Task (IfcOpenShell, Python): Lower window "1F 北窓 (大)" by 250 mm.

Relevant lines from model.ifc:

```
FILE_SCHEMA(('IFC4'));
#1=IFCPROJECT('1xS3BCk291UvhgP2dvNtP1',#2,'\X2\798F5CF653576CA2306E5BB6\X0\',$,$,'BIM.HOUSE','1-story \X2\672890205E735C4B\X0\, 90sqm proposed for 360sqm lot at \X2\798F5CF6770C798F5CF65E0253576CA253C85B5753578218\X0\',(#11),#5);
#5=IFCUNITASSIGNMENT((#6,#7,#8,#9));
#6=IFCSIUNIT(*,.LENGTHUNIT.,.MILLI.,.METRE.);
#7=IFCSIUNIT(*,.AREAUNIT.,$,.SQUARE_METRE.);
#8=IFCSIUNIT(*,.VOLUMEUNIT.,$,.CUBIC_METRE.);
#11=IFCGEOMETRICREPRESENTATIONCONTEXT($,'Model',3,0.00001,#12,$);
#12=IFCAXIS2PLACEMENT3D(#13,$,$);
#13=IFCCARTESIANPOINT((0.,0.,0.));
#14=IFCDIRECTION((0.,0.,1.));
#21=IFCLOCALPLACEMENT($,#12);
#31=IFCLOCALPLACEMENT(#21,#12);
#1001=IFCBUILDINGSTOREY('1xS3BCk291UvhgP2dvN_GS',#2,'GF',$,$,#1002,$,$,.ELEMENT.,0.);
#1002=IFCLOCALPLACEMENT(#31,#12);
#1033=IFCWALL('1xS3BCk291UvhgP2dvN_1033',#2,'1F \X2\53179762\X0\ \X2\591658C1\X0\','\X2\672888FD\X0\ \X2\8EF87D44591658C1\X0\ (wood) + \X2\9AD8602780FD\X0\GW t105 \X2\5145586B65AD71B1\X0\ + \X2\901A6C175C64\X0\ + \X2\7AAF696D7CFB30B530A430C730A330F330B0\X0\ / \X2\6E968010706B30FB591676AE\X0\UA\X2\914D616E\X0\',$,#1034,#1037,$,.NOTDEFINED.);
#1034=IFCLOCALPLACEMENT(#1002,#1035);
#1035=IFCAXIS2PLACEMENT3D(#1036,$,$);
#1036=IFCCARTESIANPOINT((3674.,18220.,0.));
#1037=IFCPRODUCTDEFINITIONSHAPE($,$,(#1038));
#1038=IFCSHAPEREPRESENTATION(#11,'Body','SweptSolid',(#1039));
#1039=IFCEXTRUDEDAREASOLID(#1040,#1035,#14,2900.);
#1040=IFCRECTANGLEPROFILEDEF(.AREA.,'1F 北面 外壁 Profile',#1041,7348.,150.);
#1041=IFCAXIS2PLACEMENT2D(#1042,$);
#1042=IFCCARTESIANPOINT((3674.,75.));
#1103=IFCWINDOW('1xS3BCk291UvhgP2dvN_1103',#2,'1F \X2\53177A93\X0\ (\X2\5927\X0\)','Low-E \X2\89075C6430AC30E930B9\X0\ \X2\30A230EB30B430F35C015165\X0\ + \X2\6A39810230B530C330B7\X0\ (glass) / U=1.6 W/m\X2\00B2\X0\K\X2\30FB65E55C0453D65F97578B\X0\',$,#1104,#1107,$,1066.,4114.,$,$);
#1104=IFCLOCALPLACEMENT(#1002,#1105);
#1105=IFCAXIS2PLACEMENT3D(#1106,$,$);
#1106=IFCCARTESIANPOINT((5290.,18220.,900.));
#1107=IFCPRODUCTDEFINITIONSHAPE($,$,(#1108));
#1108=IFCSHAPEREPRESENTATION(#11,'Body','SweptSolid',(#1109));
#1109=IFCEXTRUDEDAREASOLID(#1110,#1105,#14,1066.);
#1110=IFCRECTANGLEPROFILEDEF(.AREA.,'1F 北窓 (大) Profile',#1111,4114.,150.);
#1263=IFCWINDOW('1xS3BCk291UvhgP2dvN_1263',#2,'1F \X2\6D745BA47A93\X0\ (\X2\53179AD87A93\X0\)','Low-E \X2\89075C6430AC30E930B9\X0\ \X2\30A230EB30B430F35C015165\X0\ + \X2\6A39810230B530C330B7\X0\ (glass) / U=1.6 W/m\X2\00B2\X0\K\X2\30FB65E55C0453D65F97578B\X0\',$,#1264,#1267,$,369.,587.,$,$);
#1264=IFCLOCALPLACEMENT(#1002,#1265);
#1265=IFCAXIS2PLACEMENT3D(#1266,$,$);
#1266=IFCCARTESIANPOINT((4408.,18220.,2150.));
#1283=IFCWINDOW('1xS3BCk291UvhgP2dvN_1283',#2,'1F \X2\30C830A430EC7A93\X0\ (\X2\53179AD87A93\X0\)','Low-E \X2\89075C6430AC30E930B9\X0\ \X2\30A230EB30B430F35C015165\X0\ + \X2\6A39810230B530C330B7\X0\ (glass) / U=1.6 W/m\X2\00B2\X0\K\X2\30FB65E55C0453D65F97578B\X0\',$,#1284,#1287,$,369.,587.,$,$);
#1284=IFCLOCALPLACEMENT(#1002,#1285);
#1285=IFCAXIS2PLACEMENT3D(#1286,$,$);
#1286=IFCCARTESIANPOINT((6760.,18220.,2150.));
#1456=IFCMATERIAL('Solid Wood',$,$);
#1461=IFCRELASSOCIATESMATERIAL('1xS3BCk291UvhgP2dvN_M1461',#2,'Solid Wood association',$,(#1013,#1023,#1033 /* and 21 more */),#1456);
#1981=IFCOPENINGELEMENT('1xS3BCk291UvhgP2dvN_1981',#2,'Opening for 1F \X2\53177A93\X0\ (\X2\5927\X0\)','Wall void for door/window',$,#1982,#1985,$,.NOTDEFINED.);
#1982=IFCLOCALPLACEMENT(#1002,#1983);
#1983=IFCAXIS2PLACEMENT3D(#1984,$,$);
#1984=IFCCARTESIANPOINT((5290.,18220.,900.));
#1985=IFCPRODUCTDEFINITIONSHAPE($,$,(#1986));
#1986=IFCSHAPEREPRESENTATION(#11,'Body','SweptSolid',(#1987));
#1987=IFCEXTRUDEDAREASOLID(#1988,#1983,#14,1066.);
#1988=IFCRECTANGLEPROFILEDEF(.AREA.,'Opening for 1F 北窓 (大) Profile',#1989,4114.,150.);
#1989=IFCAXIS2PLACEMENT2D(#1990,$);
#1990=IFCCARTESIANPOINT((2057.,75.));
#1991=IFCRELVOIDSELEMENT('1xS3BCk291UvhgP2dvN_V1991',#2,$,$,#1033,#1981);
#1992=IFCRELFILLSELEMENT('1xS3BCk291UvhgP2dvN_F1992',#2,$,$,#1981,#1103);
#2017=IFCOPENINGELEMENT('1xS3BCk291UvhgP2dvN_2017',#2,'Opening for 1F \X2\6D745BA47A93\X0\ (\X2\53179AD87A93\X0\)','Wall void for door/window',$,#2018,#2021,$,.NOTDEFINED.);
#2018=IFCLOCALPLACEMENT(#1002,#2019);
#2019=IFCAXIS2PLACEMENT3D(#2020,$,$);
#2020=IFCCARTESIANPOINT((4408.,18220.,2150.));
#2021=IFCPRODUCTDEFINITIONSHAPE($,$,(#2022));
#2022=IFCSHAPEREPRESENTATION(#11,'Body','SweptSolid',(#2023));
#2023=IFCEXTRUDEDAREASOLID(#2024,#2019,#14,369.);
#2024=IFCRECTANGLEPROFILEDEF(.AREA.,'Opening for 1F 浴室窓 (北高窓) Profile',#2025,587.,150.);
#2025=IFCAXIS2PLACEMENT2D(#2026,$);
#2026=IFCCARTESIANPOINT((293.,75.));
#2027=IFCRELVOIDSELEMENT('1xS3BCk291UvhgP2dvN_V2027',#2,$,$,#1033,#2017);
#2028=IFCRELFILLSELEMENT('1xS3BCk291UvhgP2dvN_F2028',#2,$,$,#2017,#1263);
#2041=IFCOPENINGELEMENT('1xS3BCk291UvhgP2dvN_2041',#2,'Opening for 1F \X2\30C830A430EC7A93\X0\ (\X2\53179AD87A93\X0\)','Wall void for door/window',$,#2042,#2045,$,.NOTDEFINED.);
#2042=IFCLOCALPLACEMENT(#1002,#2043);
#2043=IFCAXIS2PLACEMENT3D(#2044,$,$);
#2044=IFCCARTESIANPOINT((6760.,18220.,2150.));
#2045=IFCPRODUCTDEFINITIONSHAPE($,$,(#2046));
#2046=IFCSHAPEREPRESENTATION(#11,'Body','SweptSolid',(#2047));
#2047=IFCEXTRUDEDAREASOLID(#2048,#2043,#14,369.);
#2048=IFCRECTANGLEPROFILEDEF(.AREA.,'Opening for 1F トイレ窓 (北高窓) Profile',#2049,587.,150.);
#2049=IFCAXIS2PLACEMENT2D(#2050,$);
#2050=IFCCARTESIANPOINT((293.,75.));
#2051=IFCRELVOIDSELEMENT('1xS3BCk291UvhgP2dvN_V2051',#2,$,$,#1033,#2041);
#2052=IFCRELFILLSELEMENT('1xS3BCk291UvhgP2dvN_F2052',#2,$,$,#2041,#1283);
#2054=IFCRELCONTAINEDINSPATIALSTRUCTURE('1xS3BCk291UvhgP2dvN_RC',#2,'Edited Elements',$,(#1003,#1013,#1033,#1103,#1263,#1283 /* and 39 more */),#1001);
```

```python
import numpy as np
import ifcopenshell
import ifcopenshell.api.geometry
import ifcopenshell.util.placement
import ifcopenshell.util.unit

model = ifcopenshell.open("model.ifc")
unit_scale = ifcopenshell.util.unit.calculate_unit_scale(model)

window = model.by_id(1103)
opening = window.FillsVoids[0].RelatingOpeningElement
dz = -250.0

shift = np.array([0.0, 0.0, dz])
# The window is not placed relative to its opening, so move both.
for product in (opening, window):
    matrix = ifcopenshell.util.placement.get_local_placement(product.ObjectPlacement)
    matrix[:3, 3] += shift
    ifcopenshell.api.geometry.edit_object_placement(model, product=product, matrix=matrix, is_si=False)

print(f"moved by {dz * unit_scale:+.3f} m")

model.write("model_edited.ifc")
```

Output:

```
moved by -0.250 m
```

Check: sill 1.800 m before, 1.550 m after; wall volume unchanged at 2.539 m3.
